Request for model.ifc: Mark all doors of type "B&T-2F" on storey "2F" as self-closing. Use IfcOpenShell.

First a look at what the model holds.

```python
import ifcopenshell
import ifcopenshell.util.element

model = ifcopenshell.open("model.ifc")
print(model.schema)
storey = next(s for s in model.by_type("IfcBuildingStorey") if s.Name == "2F")
doors = [e for e in ifcopenshell.util.element.get_decomposition(storey) if e.is_a("IfcDoor")]
seen = {}
for e in doors:
    element_type = ifcopenshell.util.element.get_type(e)
    key = (element_type.Name if element_type != e and element_type else None, ifcopenshell.util.element.get_pset(e, "Pset_DoorCommon", "SelfClosing"))
    seen[key] = seen.get(key, 0) + 1
for (name, value), count in sorted(seen.items(), key=str):
    print(count, "x", name, "|", value)
```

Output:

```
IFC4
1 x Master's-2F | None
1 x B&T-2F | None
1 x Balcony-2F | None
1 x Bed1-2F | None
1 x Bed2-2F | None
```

```python
import ifcopenshell
import ifcopenshell.api.pset
import ifcopenshell.util.element

model = ifcopenshell.open("model.ifc")

storey = next(s for s in model.by_type("IfcBuildingStorey") if s.Name == "2F")
doors = [e for e in ifcopenshell.util.element.get_decomposition(storey) if e.is_a("IfcDoor")]

count = 0
for e in doors:
    element_type = ifcopenshell.util.element.get_type(e)
    if element_type in (None, e) or element_type.Name != "B&T-2F":
        continue
    # add_pset returns the element's existing set when there is one.
    pset = ifcopenshell.api.pset.add_pset(model, product=e, name="Pset_DoorCommon")
    ifcopenshell.api.pset.edit_pset(model, pset=pset, properties={"SelfClosing": True})
    count += 1

print(count, "doors updated")

model.write("model_edited.ifc")
```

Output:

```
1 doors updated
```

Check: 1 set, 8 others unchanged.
